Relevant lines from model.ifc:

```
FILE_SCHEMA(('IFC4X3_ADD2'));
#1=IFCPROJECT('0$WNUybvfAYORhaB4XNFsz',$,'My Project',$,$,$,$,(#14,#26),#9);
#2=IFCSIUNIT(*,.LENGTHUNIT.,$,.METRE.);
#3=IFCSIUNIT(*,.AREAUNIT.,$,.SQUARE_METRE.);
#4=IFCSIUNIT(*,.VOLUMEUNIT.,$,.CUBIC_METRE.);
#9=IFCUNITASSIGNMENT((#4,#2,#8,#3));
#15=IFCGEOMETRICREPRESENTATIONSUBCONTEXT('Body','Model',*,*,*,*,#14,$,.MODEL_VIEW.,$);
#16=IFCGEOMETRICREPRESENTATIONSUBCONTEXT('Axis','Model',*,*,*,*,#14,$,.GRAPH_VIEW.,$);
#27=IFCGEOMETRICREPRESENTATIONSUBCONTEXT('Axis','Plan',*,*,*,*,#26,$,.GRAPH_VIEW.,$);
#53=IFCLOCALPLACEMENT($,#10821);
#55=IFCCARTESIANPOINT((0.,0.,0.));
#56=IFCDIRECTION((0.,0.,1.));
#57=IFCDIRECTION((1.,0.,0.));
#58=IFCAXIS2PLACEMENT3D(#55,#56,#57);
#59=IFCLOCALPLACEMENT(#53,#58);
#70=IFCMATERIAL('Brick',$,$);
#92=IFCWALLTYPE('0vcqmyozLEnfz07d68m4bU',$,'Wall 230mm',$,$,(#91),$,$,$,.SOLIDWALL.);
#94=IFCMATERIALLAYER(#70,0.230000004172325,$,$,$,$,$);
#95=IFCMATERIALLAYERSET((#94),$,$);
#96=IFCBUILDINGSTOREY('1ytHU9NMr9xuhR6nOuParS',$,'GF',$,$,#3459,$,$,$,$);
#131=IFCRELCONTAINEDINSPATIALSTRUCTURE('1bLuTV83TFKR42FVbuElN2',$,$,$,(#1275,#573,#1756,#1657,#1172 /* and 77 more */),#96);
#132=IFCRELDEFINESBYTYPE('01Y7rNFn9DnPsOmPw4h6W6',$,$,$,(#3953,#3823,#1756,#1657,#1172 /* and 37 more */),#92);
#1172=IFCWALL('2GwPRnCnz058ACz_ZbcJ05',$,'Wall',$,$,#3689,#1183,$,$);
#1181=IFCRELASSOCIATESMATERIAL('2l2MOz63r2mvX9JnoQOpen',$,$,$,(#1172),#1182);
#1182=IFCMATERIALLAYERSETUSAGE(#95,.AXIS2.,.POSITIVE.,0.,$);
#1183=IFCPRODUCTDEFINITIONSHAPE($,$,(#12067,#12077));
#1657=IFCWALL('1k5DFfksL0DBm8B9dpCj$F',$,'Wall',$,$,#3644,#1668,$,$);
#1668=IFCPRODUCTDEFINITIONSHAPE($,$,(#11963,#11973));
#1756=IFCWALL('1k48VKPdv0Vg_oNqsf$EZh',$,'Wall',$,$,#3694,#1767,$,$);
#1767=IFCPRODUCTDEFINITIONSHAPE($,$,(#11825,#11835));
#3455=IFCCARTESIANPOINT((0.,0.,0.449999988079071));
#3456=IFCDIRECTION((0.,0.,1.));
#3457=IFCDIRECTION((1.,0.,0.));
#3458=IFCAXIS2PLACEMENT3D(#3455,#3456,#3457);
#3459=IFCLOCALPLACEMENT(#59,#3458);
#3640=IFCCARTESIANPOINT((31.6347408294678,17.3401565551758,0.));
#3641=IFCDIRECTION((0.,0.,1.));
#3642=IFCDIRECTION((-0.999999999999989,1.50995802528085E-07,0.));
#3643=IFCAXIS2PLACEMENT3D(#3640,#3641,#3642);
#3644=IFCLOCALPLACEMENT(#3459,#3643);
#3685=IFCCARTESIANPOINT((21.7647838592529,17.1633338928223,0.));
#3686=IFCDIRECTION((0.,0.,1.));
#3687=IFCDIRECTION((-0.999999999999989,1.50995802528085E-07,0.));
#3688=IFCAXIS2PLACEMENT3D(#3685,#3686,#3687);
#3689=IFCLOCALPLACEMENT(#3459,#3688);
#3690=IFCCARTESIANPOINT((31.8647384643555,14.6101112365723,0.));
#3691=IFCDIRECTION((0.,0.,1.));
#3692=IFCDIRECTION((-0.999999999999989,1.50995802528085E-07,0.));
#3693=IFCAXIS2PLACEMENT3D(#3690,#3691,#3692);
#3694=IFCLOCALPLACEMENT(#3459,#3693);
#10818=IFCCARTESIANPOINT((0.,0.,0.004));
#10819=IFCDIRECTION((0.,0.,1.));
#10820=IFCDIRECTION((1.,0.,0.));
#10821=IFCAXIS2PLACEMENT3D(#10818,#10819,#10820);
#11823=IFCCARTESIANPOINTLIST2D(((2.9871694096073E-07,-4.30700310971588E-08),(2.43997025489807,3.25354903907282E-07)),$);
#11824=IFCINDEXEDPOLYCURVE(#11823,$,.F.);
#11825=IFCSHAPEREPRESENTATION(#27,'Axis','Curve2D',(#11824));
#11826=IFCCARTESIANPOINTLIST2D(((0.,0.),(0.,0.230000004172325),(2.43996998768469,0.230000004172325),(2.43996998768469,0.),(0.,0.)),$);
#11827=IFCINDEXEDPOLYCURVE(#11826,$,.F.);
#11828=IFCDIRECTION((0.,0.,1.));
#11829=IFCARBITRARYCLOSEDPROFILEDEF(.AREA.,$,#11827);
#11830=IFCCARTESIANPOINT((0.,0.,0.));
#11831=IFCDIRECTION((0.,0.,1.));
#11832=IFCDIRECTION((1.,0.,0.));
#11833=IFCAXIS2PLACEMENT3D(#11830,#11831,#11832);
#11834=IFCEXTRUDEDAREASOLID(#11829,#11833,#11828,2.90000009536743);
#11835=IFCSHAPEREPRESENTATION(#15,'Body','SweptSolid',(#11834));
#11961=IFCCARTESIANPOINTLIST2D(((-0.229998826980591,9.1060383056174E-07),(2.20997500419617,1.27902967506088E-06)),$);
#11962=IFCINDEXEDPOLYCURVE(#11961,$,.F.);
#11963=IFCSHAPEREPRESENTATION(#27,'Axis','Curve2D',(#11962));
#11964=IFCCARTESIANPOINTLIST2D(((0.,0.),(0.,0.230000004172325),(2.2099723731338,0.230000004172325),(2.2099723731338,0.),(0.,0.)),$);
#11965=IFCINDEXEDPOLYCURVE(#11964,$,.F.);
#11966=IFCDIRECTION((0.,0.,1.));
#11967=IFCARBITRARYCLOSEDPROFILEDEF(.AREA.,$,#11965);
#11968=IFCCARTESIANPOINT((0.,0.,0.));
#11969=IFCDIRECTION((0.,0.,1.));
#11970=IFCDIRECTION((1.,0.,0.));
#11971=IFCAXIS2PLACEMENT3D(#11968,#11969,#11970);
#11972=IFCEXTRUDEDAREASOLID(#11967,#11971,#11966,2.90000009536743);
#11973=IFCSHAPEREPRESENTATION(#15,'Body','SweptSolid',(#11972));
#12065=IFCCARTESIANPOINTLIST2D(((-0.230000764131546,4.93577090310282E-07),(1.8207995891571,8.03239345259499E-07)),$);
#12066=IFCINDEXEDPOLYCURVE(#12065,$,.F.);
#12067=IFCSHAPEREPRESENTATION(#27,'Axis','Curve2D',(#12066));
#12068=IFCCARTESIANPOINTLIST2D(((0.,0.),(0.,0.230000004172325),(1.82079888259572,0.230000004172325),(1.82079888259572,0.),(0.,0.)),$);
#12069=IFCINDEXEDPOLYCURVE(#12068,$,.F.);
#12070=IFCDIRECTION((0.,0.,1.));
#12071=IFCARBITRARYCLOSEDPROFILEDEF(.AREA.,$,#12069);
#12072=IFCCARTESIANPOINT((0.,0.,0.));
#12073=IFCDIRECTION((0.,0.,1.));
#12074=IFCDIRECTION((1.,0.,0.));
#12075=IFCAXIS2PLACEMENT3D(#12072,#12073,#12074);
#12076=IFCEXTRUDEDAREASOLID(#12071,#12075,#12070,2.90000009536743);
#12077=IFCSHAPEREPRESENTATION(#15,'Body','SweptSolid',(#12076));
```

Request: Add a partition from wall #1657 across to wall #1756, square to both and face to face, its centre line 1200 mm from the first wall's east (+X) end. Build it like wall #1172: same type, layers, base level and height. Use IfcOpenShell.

```python
import numpy as np
import ifcopenshell
import ifcopenshell.api.geometry
import ifcopenshell.api.material
import ifcopenshell.api.pset
import ifcopenshell.api.root
import ifcopenshell.api.spatial
import ifcopenshell.api.type
import ifcopenshell.geom
import ifcopenshell.util.element
import ifcopenshell.util.placement
import ifcopenshell.util.representation
import ifcopenshell.util.shape
import ifcopenshell.util.unit

model = ifcopenshell.open("model.ifc")
unit_scale = ifcopenshell.util.unit.calculate_unit_scale(model)
settings = ifcopenshell.geom.settings()
settings.set("use-world-coords", True)

start_wall = model.by_id(1657)
end_wall = model.by_guid("1k48VKPdv0Vg_oNqsf$EZh")
like = model.by_guid("2GwPRnCnz058ACz_ZbcJ05")
matrix = ifcopenshell.util.placement.get_local_placement(start_wall.ObjectPlacement)
matrix[:3, 3] *= unit_scale


def extent(element):
    """Bounding box in the first wall's axes, in metres."""
    shape = ifcopenshell.geom.create_shape(settings, element)
    points = (ifcopenshell.util.shape.get_vertices(shape.geometry) - matrix[:3, 3]) @ matrix[:3, :3]
    return points.min(axis=0), points.max(axis=0)


y_start = extent(start_wall)[1][1]
y_end = extent(end_wall)[0][1]
like_min, like_max = extent(like)
length, height = float(abs(y_end - y_start)), float(like_max[2] - like_min[2])
layer_set = ifcopenshell.util.element.get_material(like, should_skip_usage=True)
thickness = sum(layer.LayerThickness for layer in layer_set.MaterialLayers) * unit_scale

wall = ifcopenshell.api.root.create_entity(model, ifc_class="IfcWall", name="New partition")
storey = ifcopenshell.util.element.get_container(like)
ifcopenshell.api.spatial.assign_container(model, products=[wall], relating_structure=storey)
ifcopenshell.api.type.assign_type(
    model, related_objects=[wall], relating_type=ifcopenshell.util.element.get_type(like), should_map_representations=False
)
rel = ifcopenshell.api.material.assign_material(
    model, products=[wall], type="IfcMaterialLayerSetUsage", material=layer_set
)
rel.RelatingMaterial.OffsetFromReferenceLine = -thickness / 2 / unit_scale
pset = ifcopenshell.api.pset.add_pset(model, product=wall, name="Pset_WallCommon")
ifcopenshell.api.pset.edit_pset(model, pset=pset, properties={"IsExternal": False, "LoadBearing": False})

# The axis runs down the middle of the wall.
axis = ifcopenshell.api.geometry.add_axis_representation(
    model, context=ifcopenshell.util.representation.get_context(model, "Model", "Axis"), axis=[(0.0, 0.0), (length, 0.0)]
)
body = ifcopenshell.api.geometry.add_wall_representation(
    model,
    context=ifcopenshell.util.representation.get_context(model, "Model", "Body", "MODEL_VIEW"),
    length=length,
    height=height,
    thickness=thickness,
    offset=-thickness / 2,
)
for representation in (axis, body):
    ifcopenshell.api.geometry.assign_representation(model, product=wall, representation=representation)

placement = matrix @ ifcopenshell.util.placement.rotation(90, "Z")
placement[:, 3] = matrix @ np.array([extent(start_wall)[0][0] + 1.2, y_start, like_min[2], 1.0])
ifcopenshell.api.geometry.edit_object_placement(model, product=wall, matrix=placement)

print(f"partition {length:.3f} m long, {height:.3f} m high, {thickness:.3f} m thick")

model.write("model_rev.ifc")
```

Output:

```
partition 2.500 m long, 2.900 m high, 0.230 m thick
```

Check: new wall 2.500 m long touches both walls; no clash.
